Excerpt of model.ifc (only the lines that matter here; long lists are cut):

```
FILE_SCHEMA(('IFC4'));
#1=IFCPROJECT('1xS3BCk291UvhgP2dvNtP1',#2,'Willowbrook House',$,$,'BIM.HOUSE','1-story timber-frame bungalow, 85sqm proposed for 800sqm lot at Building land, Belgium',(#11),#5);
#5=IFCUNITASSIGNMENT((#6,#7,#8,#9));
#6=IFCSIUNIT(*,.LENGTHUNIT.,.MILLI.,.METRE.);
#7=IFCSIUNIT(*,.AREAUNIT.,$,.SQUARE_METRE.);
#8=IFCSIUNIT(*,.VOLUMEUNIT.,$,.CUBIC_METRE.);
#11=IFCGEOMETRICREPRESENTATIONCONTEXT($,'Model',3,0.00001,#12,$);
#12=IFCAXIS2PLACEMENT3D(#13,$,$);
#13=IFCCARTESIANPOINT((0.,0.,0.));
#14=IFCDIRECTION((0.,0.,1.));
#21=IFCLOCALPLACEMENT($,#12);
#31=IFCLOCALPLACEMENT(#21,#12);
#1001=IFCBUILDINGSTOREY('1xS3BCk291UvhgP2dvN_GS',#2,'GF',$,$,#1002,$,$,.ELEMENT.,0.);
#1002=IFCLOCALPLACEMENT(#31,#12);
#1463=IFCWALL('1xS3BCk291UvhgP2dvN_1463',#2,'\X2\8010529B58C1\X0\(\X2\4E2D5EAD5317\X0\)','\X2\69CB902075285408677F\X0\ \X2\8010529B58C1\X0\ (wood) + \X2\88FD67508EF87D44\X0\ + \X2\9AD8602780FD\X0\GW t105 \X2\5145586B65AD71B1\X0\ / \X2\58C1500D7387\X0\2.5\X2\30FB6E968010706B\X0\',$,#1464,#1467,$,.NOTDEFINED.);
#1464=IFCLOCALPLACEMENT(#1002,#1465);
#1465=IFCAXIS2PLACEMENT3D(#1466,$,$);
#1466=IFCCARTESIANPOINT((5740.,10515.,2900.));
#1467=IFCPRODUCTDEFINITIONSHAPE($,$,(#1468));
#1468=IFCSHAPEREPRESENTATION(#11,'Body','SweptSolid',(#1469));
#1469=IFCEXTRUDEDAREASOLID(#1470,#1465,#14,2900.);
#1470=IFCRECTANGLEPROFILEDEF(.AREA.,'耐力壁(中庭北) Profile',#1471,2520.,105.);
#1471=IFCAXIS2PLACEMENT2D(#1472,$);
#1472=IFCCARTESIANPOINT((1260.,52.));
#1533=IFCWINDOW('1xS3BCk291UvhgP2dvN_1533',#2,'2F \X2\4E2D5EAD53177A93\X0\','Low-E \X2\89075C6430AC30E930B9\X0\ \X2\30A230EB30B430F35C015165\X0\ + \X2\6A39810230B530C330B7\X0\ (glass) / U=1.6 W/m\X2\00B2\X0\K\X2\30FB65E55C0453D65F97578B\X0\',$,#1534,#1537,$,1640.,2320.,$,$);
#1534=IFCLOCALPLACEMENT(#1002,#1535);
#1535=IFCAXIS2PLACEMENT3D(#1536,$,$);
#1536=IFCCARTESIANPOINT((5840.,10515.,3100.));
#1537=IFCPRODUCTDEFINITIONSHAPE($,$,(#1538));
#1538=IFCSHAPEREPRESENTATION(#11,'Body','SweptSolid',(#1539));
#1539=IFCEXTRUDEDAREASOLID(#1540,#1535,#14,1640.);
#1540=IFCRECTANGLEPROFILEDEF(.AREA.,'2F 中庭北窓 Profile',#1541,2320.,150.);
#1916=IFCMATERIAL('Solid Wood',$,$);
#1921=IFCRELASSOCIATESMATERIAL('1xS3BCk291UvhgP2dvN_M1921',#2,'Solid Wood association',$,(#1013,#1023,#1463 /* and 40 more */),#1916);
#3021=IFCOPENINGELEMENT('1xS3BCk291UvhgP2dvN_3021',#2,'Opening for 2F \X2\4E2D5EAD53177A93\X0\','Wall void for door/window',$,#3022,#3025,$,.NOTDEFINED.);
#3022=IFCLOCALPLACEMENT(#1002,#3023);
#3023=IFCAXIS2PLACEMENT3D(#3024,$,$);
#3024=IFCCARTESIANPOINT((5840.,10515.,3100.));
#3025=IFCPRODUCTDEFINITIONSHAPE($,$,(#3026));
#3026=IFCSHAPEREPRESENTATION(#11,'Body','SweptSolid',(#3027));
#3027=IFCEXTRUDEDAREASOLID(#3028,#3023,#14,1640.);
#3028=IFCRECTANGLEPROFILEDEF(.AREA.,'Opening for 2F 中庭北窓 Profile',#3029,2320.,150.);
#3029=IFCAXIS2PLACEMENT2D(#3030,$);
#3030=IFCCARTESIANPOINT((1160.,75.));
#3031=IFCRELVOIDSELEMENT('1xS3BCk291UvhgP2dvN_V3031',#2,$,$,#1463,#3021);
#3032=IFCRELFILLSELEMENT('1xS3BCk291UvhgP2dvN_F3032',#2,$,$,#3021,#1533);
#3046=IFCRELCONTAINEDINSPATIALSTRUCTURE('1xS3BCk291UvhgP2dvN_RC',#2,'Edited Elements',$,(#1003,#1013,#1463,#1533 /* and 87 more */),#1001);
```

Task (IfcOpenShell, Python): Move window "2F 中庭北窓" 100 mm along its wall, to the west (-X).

```python
import ifcopenshell
import ifcopenshell.api.geometry
import ifcopenshell.util.placement
import ifcopenshell.util.unit

model = ifcopenshell.open("model.ifc")
unit_scale = ifcopenshell.util.unit.calculate_unit_scale(model)

window = model.by_guid("1xS3BCk291UvhgP2dvN_1533")
opening = window.FillsVoids[0].RelatingOpeningElement
wall = opening.VoidsElements[0].RelatingBuildingElement

wall_matrix = ifcopenshell.util.placement.get_local_placement(wall.ObjectPlacement)
shift = wall_matrix[:3, 0] * -0.1 / unit_scale
before = ifcopenshell.util.placement.get_local_placement(window.ObjectPlacement)[:3, 3].copy()

# The window is not placed relative to its opening, so move both.
for product in (opening, window):
    matrix = ifcopenshell.util.placement.get_local_placement(product.ObjectPlacement)
    matrix[:3, 3] += shift
    ifcopenshell.api.geometry.edit_object_placement(model, product=product, matrix=matrix, is_si=False)

after = ifcopenshell.util.placement.get_local_placement(window.ObjectPlacement)[:3, 3]
print("window moved by", (after - before).round(3) + 0.0)

model.write("model_v2.ifc")
```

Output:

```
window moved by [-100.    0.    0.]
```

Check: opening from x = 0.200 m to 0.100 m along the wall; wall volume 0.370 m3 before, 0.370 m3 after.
